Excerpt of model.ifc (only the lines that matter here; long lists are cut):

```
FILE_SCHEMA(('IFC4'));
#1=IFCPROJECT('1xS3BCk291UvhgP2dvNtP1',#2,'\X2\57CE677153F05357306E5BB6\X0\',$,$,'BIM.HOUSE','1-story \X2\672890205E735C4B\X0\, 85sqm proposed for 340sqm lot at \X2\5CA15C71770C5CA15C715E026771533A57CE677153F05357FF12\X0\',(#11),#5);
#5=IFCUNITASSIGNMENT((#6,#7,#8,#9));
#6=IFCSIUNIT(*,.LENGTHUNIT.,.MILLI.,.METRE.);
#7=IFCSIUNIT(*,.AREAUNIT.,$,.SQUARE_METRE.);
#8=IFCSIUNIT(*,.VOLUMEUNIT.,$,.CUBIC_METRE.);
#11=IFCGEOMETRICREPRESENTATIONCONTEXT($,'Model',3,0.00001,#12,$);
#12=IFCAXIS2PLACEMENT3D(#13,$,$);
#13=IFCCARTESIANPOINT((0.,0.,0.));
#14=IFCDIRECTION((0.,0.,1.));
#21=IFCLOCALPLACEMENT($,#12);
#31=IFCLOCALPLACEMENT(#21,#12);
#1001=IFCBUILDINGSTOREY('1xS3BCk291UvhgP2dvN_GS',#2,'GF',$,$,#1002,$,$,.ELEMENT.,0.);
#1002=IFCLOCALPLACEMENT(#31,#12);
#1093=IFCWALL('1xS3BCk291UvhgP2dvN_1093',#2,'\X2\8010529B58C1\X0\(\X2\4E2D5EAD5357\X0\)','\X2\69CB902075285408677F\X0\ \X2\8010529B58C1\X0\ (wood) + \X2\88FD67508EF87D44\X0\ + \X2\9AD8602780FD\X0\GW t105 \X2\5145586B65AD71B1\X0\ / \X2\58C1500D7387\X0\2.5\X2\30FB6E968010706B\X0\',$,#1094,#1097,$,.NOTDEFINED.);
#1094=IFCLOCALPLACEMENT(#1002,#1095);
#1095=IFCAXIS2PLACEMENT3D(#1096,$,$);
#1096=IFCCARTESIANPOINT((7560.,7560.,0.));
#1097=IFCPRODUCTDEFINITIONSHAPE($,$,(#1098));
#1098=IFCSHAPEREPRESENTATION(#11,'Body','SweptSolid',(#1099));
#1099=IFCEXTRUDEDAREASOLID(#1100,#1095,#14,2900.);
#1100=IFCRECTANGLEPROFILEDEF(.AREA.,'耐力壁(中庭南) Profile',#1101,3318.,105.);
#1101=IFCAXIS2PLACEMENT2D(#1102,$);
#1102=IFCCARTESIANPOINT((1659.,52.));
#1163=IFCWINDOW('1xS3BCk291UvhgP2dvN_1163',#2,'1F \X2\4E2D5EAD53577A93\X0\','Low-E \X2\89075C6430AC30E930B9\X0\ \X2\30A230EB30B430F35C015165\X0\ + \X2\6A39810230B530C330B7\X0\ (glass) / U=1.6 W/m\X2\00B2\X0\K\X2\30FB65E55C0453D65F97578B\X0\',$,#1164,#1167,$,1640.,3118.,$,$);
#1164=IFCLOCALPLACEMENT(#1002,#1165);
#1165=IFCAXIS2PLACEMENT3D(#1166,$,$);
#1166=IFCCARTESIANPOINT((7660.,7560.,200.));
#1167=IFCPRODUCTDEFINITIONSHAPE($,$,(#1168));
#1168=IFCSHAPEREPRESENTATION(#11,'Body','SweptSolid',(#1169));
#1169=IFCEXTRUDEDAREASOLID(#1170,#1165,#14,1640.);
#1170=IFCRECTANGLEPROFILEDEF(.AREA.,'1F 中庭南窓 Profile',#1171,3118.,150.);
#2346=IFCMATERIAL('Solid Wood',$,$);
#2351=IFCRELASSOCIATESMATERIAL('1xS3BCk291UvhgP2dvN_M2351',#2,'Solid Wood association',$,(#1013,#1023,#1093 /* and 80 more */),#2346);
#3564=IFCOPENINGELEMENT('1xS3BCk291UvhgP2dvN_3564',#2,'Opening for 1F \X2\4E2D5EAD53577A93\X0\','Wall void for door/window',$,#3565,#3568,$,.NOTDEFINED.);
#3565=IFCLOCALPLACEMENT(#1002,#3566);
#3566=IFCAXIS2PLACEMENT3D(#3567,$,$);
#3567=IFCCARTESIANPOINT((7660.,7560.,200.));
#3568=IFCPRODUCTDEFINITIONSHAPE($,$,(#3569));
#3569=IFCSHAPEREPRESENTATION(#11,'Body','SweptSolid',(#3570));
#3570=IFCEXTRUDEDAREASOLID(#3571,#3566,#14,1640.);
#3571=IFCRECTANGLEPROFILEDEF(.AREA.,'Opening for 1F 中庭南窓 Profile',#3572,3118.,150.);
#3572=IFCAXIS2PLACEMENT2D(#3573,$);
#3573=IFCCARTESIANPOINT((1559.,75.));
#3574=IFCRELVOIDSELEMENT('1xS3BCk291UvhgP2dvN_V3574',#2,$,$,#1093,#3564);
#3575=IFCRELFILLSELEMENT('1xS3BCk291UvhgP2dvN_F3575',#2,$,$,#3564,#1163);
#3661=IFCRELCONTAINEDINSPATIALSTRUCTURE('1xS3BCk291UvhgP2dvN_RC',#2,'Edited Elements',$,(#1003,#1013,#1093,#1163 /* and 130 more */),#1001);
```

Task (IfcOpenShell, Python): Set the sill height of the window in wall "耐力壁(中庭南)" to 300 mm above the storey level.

```python
import numpy as np
import ifcopenshell
import ifcopenshell.api.geometry
import ifcopenshell.geom
import ifcopenshell.util.element
import ifcopenshell.util.placement
import ifcopenshell.util.shape
import ifcopenshell.util.unit

model = ifcopenshell.open("model.ifc")
unit_scale = ifcopenshell.util.unit.calculate_unit_scale(model)

window = model.by_id(1163)
opening = window.FillsVoids[0].RelatingOpeningElement
storey = ifcopenshell.util.element.get_container(window, ifc_class="IfcBuildingStorey")
level = ifcopenshell.util.placement.get_local_placement(storey.ObjectPlacement)[2, 3]

# The opening's origin need not be at the sill, so measure its lowest point.
shape = ifcopenshell.geom.create_shape(ifcopenshell.geom.settings(), opening)
bottom = ifcopenshell.util.shape.get_shape_bottom_elevation(shape, shape.geometry) / unit_scale
dz = level + 0.3 / unit_scale - bottom

shift = np.array([0.0, 0.0, dz])
# The window is not placed relative to its opening, so move both.
for product in (opening, window):
    matrix = ifcopenshell.util.placement.get_local_placement(product.ObjectPlacement)
    matrix[:3, 3] += shift
    ifcopenshell.api.geometry.edit_object_placement(model, product=product, matrix=matrix, is_si=False)

print(f"moved by {dz * unit_scale:+.3f} m")

model.write("model-out.ifc")
```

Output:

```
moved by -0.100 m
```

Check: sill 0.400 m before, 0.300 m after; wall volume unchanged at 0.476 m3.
